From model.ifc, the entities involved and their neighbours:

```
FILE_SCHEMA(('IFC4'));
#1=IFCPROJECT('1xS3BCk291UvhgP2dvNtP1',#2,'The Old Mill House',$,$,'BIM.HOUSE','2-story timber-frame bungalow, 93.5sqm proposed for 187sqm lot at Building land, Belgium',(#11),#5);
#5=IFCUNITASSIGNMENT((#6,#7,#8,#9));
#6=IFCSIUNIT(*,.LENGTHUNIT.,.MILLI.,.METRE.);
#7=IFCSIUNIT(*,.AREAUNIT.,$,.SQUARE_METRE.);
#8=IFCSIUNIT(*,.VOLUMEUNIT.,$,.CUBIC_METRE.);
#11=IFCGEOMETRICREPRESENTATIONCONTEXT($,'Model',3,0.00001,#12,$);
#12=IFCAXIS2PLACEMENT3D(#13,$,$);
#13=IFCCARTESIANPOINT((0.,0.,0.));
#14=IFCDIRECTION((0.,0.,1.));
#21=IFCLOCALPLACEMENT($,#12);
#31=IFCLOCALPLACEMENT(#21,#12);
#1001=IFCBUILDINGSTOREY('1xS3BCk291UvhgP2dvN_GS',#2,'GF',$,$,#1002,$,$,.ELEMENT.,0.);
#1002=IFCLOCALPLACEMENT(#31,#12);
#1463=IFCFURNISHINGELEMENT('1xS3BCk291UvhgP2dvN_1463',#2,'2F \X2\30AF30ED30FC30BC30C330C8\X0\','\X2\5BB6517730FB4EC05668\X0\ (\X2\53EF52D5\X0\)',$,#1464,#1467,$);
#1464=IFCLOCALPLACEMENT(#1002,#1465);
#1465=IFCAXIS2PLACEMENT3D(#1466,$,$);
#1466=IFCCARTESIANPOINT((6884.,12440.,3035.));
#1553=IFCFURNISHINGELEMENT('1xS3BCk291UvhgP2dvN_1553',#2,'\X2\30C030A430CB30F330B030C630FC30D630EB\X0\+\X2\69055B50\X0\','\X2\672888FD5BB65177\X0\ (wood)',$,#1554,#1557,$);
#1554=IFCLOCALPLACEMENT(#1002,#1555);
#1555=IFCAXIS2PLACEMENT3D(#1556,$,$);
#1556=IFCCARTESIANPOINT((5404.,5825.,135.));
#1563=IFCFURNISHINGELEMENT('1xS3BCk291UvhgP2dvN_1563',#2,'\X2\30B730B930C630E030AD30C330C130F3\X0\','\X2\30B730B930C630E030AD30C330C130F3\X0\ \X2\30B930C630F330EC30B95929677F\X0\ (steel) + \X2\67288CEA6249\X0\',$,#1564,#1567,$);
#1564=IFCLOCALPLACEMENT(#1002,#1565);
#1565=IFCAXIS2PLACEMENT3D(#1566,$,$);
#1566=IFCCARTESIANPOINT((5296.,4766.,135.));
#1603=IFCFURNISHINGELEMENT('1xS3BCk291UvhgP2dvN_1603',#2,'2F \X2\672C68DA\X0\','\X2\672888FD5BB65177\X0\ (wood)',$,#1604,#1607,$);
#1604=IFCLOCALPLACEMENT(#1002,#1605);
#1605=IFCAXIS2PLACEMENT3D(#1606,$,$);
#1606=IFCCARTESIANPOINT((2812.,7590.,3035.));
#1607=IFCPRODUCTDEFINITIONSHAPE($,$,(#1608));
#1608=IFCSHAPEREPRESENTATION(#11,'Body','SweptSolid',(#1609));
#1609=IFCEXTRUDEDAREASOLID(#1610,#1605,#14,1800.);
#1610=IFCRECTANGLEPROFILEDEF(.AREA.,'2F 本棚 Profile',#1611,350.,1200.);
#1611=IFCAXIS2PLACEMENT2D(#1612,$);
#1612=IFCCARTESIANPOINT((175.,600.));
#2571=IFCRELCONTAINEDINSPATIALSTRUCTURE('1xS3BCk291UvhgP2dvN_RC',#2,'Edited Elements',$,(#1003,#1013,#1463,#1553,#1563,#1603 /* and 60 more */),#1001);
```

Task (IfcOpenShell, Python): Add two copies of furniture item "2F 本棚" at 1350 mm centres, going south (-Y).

```python
import numpy as np
import ifcopenshell
import ifcopenshell.api.geometry
import ifcopenshell.api.root
import ifcopenshell.util.element
import ifcopenshell.util.placement
import ifcopenshell.util.unit

model = ifcopenshell.open("model.ifc")
unit_scale = ifcopenshell.util.unit.calculate_unit_scale(model)


def reuse_history(source, copy):
    """copy_class also copies each property set's owner history, people and application; keep the originals."""
    for rel in copy.IsDefinedBy:
        if rel.is_a("IfcRelDefinesByProperties") and (history := rel.RelatingPropertyDefinition.OwnerHistory):
            rel.RelatingPropertyDefinition.OwnerHistory = source.OwnerHistory
            ifcopenshell.util.element.remove_deep2(model, history)


source = model.by_id(1603)
base = ifcopenshell.util.placement.get_local_placement(source.ObjectPlacement)
step = np.array([0.0, -1.0, 0.0]) * 1.35 / unit_scale

for i in range(1, 3):
    copy = ifcopenshell.api.root.copy_class(model, product=source)
    copy.Representation = ifcopenshell.util.element.copy_deep(
        model, source.Representation, exclude=["IfcGeometricRepresentationContext", "IfcRepresentationMap"]
    )
    reuse_history(source, copy)
    matrix = base.copy()
    matrix[:3, 3] += i * step
    print("added at", matrix[:3, 3].round(3) + 0.0)
    ifcopenshell.api.geometry.edit_object_placement(model, product=copy, matrix=matrix, is_si=False)

model.write("model-out.ifc")
```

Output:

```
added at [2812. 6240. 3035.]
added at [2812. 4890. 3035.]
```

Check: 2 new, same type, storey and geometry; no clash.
